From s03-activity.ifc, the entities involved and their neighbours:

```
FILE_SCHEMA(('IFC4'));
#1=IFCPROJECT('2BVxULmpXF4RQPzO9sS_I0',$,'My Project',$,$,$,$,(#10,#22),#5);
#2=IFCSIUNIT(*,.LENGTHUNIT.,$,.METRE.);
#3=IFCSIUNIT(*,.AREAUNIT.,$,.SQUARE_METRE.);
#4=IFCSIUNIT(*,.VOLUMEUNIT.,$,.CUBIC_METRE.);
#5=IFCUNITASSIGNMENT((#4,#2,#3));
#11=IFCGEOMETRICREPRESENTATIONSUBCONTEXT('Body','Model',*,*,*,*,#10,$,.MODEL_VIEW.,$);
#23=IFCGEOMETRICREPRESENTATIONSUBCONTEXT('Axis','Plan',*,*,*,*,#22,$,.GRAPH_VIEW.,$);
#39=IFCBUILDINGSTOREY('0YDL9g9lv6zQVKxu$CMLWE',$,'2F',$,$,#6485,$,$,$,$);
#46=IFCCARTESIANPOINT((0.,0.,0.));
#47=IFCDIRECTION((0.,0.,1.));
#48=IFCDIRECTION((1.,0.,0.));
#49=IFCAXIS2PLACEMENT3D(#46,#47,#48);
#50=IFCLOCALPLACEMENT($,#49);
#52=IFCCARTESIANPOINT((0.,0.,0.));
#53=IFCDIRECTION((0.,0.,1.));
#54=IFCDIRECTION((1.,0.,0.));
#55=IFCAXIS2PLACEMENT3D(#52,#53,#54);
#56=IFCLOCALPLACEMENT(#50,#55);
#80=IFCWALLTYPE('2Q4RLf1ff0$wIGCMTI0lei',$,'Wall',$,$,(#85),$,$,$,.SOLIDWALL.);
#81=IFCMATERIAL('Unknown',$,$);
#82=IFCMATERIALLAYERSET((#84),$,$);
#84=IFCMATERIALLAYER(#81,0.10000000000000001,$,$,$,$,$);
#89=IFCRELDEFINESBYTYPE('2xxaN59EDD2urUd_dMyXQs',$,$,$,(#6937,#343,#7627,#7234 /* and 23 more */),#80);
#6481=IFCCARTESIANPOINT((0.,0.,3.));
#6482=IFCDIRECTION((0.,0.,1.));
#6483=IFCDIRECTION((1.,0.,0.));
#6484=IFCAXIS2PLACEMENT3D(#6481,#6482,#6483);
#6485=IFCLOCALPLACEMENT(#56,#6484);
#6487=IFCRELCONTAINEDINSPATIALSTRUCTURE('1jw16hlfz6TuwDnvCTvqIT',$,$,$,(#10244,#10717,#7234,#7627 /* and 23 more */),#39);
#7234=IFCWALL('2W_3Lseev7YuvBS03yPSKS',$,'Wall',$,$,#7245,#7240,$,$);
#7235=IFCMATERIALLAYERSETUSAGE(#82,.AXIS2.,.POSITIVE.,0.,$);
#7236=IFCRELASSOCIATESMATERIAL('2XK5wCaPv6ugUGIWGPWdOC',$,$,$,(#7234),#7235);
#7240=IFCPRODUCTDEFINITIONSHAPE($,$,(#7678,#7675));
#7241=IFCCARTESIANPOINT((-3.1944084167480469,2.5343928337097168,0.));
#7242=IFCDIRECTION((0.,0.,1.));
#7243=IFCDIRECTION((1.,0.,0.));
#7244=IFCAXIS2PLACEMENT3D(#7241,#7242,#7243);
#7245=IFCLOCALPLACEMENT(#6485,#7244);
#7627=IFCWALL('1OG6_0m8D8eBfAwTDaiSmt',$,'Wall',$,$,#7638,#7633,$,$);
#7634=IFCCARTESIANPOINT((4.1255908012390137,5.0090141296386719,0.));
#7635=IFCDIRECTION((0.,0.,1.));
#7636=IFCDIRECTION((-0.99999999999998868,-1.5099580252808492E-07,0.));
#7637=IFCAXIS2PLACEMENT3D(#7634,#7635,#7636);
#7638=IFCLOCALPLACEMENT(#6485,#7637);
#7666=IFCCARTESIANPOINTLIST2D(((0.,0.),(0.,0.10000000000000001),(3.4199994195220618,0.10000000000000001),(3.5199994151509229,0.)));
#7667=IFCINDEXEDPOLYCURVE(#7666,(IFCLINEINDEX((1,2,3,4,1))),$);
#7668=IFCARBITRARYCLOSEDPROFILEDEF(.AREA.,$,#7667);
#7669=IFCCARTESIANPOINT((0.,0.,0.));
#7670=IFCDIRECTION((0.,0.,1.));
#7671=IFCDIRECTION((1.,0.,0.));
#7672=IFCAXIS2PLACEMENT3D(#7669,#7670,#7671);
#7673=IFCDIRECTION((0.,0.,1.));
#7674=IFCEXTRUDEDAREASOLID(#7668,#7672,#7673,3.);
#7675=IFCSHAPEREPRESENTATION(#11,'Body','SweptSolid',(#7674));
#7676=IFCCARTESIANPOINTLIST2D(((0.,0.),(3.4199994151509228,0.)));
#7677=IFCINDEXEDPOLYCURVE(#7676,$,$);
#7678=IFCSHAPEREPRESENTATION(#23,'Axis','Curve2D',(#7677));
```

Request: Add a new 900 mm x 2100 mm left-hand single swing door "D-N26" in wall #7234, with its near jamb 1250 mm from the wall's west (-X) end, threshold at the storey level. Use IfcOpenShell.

```python
import numpy as np
import ifcopenshell
import ifcopenshell.api.feature
import ifcopenshell.api.geometry
import ifcopenshell.api.root
import ifcopenshell.api.spatial
import ifcopenshell.geom
import ifcopenshell.util.element
import ifcopenshell.util.placement
import ifcopenshell.util.representation
import ifcopenshell.util.shape
import ifcopenshell.util.unit

model = ifcopenshell.open("s03-activity.ifc")
unit_scale = ifcopenshell.util.unit.calculate_unit_scale(model)
settings = ifcopenshell.geom.settings()


def volume(element):
    """Net volume in cubic metres, openings subtracted."""
    shape = ifcopenshell.geom.create_shape(settings, element)
    return ifcopenshell.util.shape.get_volume(shape.geometry)


wall = model.by_guid("2W_3Lseev7YuvBS03yPSKS")
storey = ifcopenshell.util.element.get_container(wall, ifc_class="IfcBuildingStorey")
context = ifcopenshell.util.representation.get_context(model, "Model", "Body", "MODEL_VIEW")
before = volume(wall)

width, height, from_end, sill = 0.9, 2.1, 1.25, 0.0  # metres

# The wall runs along its own X axis, and the end named is its -X end.
wall_shape = ifcopenshell.geom.create_shape(settings, wall)
x, y, z = ifcopenshell.util.shape.get_vertices(wall_shape.geometry).T
start = x.min() + from_end
face, thickness = float(y.min()), float(y.max() - y.min())
wall_matrix = ifcopenshell.util.placement.get_local_placement(wall.ObjectPlacement)
level = ifcopenshell.util.placement.get_local_placement(storey.ObjectPlacement)[2, 3]


def in_wall(x, y):
    """Placement at x, y metres in the wall's axes, at sill height."""
    matrix = wall_matrix.copy()
    matrix[:, 3] = wall_matrix @ np.array([x / unit_scale, y / unit_scale, 0.0, 1.0])
    matrix[2, 3] = level + sill / unit_scale
    return matrix


# Opening: a box that overshoots both wall faces by 50 mm.
opening = ifcopenshell.api.root.create_entity(model, ifc_class="IfcOpeningElement", predefined_type="OPENING")
box = ifcopenshell.api.geometry.add_wall_representation(
    model, context=context, length=width, height=height, thickness=thickness + 0.1
)
ifcopenshell.api.geometry.assign_representation(model, product=opening, representation=box)
ifcopenshell.api.geometry.edit_object_placement(model, product=opening, matrix=in_wall(start, face - 0.05), is_si=False)
ifcopenshell.api.feature.add_feature(model, feature=opening, element=wall)

door = ifcopenshell.api.root.create_entity(model, ifc_class="IfcDoor", name="D-N26", predefined_type="DOOR")
door.OverallWidth, door.OverallHeight = width / unit_scale, height / unit_scale
door.OperationType = "SINGLE_SWING_LEFT"
body = ifcopenshell.api.geometry.add_door_representation(
    model,
    context=context,
    overall_width=door.OverallWidth,
    overall_height=door.OverallHeight,
    operation_type="SINGLE_SWING_LEFT",
    lining_properties={"LiningDepth": thickness / unit_scale, "ThresholdDepth": thickness / unit_scale},
)
ifcopenshell.api.geometry.assign_representation(model, product=door, representation=body)
ifcopenshell.api.spatial.assign_container(model, products=[door], relating_structure=storey)
ifcopenshell.api.feature.add_filling(model, opening=opening, element=door)

# The lining spans the wall, so the door starts at the wall face.
ifcopenshell.api.geometry.edit_object_placement(model, product=door, matrix=in_wall(start, face), is_si=False)

after = volume(wall)

print(f"wall volume {before:.3f} -> {after:.3f} m3")

model.write("s03-activity_updated.ifc")
```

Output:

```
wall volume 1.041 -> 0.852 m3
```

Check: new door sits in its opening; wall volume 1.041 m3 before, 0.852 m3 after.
